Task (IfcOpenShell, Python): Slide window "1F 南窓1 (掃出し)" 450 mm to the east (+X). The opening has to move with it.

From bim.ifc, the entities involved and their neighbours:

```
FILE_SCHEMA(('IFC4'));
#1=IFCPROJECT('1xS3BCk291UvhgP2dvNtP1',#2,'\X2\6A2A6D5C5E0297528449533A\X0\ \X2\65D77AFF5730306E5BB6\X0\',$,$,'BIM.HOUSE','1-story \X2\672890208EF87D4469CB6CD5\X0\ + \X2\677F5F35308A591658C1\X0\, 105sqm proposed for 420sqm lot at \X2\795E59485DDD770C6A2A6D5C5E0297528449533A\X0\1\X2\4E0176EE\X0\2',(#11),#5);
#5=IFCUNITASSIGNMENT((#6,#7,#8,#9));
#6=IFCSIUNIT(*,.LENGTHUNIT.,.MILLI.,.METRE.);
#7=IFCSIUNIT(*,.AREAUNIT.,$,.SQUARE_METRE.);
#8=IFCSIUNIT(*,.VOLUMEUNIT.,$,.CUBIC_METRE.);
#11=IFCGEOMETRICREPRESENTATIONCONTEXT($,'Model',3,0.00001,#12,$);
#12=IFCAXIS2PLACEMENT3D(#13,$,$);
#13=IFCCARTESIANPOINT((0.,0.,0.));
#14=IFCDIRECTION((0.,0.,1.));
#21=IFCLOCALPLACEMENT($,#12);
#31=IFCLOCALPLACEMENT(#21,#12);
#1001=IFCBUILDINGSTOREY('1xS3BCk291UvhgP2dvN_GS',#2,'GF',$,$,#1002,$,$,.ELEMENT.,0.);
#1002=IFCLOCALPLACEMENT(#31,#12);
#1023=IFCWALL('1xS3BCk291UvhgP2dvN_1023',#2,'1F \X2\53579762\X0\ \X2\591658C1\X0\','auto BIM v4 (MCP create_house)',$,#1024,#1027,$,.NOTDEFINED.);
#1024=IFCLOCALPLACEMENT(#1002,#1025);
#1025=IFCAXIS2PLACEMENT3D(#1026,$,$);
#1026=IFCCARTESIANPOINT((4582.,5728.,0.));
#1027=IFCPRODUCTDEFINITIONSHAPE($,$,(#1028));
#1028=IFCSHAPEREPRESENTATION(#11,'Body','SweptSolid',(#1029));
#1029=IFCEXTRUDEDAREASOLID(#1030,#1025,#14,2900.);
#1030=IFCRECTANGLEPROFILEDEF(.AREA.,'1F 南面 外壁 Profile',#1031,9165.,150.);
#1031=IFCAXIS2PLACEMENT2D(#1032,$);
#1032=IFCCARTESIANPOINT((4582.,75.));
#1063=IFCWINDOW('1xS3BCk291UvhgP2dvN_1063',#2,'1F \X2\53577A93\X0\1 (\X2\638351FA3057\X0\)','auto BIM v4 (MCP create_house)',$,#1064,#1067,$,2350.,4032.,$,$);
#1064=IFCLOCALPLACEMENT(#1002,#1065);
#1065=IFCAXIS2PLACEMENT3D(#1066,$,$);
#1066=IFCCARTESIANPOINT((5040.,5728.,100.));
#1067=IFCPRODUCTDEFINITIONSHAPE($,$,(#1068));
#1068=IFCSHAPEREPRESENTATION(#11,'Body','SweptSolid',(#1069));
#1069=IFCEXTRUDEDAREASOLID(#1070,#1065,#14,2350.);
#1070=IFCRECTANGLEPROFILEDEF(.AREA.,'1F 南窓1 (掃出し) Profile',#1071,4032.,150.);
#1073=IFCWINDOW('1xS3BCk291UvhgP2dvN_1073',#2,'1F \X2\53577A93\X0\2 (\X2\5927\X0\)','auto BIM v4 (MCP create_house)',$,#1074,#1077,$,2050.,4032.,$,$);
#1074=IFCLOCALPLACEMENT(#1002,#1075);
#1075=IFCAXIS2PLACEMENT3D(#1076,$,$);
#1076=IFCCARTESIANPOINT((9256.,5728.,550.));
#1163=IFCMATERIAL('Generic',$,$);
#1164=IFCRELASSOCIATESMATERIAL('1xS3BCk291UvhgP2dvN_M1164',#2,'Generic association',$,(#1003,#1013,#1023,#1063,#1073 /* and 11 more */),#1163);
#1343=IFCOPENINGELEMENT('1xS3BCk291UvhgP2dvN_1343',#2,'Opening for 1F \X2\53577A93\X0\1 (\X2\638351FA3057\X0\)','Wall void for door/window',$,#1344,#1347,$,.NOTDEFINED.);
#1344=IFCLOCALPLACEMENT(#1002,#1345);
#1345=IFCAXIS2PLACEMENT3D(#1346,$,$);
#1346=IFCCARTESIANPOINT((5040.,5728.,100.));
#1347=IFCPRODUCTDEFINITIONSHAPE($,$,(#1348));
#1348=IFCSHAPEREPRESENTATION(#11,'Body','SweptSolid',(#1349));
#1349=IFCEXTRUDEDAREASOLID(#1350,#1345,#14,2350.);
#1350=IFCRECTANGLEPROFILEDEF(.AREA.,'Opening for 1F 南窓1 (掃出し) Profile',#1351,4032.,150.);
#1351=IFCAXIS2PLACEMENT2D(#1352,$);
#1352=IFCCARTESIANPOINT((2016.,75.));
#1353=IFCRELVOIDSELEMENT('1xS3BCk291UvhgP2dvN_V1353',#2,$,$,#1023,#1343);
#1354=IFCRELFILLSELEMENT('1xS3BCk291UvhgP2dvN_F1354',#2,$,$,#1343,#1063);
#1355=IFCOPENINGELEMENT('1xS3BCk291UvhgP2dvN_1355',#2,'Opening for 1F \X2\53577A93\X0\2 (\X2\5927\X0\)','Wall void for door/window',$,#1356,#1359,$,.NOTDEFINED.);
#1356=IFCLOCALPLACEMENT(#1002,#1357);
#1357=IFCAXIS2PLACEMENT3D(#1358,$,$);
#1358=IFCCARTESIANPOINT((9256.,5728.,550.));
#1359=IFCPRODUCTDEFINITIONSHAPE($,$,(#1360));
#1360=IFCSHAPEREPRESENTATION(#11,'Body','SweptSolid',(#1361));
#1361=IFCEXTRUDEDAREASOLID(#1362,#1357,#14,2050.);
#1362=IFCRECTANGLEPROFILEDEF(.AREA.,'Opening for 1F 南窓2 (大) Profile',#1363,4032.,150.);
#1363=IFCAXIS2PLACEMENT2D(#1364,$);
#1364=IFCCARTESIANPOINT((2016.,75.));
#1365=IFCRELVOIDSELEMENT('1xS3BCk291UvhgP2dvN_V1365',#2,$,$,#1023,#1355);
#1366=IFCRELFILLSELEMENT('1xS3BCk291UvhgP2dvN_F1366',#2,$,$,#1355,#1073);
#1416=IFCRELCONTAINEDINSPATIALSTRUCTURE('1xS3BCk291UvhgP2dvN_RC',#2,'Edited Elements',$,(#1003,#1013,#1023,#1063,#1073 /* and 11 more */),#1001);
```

```python
import ifcopenshell
import ifcopenshell.api.geometry
import ifcopenshell.util.placement
import ifcopenshell.util.unit

model = ifcopenshell.open("bim.ifc")
unit_scale = ifcopenshell.util.unit.calculate_unit_scale(model)

window = model.by_id(1063)
opening = window.FillsVoids[0].RelatingOpeningElement
wall = opening.VoidsElements[0].RelatingBuildingElement

wall_matrix = ifcopenshell.util.placement.get_local_placement(wall.ObjectPlacement)
shift = wall_matrix[:3, 0] * 0.45 / unit_scale
before = ifcopenshell.util.placement.get_local_placement(window.ObjectPlacement)[:3, 3].copy()

# The window is not placed relative to its opening, so move both.
for product in (opening, window):
    matrix = ifcopenshell.util.placement.get_local_placement(product.ObjectPlacement)
    matrix[:3, 3] += shift
    ifcopenshell.api.geometry.edit_object_placement(model, product=product, matrix=matrix, is_si=False)

after = ifcopenshell.util.placement.get_local_placement(window.ObjectPlacement)[:3, 3]
print("window moved by", (after - before).round(3) + 0.0)

model.write("bim_v2.ifc")
```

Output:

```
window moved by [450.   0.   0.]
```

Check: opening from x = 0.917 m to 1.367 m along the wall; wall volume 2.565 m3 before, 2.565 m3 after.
